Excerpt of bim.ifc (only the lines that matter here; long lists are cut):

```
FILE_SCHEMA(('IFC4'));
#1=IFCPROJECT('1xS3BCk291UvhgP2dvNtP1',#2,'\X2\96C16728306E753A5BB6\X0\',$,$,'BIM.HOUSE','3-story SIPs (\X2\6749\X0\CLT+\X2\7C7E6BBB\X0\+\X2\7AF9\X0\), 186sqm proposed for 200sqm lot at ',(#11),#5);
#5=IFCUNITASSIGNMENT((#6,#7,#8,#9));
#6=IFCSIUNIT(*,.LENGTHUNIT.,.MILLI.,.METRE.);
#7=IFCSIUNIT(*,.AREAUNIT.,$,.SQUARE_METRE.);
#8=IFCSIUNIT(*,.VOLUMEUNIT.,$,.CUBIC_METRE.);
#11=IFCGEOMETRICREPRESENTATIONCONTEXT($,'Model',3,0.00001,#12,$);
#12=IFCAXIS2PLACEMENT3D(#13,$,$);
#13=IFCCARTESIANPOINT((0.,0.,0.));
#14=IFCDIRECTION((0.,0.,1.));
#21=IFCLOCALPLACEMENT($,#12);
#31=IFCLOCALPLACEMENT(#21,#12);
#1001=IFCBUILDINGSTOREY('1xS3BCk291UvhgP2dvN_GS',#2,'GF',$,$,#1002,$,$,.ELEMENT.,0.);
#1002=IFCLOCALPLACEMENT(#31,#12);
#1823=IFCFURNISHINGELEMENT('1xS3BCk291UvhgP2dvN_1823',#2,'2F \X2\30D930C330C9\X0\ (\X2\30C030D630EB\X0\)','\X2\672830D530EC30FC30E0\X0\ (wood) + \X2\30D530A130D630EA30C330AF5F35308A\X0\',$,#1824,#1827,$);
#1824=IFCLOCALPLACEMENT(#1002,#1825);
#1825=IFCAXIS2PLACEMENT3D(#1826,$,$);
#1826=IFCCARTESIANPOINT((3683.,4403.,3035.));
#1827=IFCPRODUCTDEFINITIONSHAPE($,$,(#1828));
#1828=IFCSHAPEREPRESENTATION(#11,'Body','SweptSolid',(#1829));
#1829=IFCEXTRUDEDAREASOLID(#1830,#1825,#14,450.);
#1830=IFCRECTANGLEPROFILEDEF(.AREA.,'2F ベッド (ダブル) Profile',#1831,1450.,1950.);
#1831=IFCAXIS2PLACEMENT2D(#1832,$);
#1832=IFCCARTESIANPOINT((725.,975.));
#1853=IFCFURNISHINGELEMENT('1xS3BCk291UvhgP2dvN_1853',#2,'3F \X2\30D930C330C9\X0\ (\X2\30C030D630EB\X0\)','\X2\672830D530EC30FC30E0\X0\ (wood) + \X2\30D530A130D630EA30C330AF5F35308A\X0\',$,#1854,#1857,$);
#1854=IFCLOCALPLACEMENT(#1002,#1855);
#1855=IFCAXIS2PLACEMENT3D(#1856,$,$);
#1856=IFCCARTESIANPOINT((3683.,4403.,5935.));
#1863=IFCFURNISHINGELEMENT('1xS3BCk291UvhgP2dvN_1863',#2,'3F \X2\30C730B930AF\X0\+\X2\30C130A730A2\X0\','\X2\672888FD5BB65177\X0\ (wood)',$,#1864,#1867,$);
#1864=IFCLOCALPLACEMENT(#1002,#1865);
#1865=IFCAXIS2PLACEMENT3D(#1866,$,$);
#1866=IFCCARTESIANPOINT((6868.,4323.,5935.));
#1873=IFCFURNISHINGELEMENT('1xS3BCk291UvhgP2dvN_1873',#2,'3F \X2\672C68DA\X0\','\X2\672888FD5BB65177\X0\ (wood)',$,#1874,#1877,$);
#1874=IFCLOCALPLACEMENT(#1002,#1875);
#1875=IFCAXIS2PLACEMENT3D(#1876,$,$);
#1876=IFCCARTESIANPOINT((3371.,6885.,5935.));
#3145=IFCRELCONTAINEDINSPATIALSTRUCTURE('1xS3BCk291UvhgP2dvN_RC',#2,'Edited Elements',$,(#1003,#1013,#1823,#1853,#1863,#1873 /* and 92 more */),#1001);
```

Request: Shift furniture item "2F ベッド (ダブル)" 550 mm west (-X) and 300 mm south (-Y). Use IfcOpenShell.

```python
import ifcopenshell
import ifcopenshell.api.geometry
import ifcopenshell.util.placement
import ifcopenshell.util.unit

model = ifcopenshell.open("bim.ifc")
unit_scale = ifcopenshell.util.unit.calculate_unit_scale(model)

item = model.by_guid("1xS3BCk291UvhgP2dvN_1823")
matrix = ifcopenshell.util.placement.get_local_placement(item.ObjectPlacement)
matrix[0, 3] -= 0.55 / unit_scale
matrix[1, 3] -= 0.3 / unit_scale
ifcopenshell.api.geometry.edit_object_placement(model, product=item, matrix=matrix, is_si=False)

print(ifcopenshell.util.placement.get_local_placement(item.ObjectPlacement).round(3) + 0.0)

model.write("bim_v2.ifc")
```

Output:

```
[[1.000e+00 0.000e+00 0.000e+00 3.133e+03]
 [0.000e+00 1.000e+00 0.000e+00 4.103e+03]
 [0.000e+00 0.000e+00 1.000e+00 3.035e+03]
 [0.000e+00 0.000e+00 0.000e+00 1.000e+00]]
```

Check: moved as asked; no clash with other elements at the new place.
